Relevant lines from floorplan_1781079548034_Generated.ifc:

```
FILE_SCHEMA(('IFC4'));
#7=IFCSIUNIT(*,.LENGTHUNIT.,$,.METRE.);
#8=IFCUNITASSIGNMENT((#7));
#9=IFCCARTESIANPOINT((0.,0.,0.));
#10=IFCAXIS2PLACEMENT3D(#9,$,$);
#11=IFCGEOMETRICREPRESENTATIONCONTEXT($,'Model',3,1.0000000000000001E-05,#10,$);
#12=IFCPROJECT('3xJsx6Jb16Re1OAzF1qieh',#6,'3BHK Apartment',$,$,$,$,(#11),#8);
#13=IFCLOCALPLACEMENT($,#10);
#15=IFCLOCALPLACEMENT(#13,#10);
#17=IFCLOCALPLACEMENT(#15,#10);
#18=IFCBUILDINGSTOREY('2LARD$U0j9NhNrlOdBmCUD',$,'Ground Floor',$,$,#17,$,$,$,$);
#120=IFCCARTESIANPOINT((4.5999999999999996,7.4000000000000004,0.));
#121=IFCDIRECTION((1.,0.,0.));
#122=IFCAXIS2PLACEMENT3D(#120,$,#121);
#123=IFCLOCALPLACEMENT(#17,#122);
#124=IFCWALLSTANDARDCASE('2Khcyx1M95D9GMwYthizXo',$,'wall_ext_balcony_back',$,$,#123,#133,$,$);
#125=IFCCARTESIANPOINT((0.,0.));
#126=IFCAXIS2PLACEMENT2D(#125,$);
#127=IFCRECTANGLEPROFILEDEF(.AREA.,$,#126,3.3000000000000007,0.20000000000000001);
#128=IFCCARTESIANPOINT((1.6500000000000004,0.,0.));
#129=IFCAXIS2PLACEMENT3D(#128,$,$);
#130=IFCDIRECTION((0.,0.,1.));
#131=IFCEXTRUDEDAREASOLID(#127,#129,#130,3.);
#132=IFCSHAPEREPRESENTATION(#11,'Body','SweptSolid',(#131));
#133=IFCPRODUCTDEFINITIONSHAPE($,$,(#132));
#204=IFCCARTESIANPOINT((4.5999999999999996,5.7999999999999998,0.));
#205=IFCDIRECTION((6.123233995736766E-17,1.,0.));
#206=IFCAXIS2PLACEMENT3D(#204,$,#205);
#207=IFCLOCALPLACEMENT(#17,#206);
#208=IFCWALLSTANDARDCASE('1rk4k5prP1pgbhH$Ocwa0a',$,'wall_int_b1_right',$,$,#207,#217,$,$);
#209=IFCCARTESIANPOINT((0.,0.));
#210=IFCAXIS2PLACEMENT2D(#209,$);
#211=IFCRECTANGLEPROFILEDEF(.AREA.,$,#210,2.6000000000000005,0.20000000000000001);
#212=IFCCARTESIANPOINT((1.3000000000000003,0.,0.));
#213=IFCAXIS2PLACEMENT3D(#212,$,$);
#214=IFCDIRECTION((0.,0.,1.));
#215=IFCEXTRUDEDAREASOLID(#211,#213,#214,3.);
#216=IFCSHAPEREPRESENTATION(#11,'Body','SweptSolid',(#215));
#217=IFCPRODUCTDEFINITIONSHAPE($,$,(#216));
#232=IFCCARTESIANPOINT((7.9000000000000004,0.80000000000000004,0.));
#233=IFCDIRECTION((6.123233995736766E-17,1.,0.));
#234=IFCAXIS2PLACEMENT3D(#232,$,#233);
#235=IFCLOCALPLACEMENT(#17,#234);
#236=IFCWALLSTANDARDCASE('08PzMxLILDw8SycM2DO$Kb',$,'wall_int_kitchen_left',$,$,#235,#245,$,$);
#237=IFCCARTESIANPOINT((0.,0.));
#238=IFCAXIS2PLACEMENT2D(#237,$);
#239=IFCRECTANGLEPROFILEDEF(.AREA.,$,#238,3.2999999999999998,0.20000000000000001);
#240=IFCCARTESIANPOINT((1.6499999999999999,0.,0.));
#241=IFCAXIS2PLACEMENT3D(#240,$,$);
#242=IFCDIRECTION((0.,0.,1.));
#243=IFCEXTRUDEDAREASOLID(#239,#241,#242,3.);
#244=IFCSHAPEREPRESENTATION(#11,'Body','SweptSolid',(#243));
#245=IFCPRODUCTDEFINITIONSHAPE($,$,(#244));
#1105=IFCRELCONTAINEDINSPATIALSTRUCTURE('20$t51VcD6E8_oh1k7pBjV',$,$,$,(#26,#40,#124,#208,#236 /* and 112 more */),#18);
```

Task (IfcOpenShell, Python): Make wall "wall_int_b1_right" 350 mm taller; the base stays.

```python
import ifcopenshell
import ifcopenshell.geom
import ifcopenshell.util.shape
import ifcopenshell.util.unit

model = ifcopenshell.open("floorplan_1781079548034_Generated.ifc")
unit_scale = ifcopenshell.util.unit.calculate_unit_scale(model)
settings = ifcopenshell.geom.settings()


def volume(element):
    """Net volume in cubic metres, openings subtracted."""
    shape = ifcopenshell.geom.create_shape(settings, element)
    return ifcopenshell.util.shape.get_volume(shape.geometry)


wall = model.by_guid("1rk4k5prP1pgbhH$Ocwa0a")
before = volume(wall)

body = next(r for r in wall.Representation.Representations if r.RepresentationIdentifier == "Body")
solid = body.Items[0]
old_height = solid.Depth
solid.Depth += 0.35 / unit_scale
after = volume(wall)

print(f"height {old_height:g} -> {solid.Depth:g}, volume {before:.3f} -> {after:.3f} m3")

model.write("floorplan_1781079548034_Generated_updated.ifc")
```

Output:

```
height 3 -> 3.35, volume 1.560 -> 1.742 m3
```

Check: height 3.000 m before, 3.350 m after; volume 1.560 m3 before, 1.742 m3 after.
